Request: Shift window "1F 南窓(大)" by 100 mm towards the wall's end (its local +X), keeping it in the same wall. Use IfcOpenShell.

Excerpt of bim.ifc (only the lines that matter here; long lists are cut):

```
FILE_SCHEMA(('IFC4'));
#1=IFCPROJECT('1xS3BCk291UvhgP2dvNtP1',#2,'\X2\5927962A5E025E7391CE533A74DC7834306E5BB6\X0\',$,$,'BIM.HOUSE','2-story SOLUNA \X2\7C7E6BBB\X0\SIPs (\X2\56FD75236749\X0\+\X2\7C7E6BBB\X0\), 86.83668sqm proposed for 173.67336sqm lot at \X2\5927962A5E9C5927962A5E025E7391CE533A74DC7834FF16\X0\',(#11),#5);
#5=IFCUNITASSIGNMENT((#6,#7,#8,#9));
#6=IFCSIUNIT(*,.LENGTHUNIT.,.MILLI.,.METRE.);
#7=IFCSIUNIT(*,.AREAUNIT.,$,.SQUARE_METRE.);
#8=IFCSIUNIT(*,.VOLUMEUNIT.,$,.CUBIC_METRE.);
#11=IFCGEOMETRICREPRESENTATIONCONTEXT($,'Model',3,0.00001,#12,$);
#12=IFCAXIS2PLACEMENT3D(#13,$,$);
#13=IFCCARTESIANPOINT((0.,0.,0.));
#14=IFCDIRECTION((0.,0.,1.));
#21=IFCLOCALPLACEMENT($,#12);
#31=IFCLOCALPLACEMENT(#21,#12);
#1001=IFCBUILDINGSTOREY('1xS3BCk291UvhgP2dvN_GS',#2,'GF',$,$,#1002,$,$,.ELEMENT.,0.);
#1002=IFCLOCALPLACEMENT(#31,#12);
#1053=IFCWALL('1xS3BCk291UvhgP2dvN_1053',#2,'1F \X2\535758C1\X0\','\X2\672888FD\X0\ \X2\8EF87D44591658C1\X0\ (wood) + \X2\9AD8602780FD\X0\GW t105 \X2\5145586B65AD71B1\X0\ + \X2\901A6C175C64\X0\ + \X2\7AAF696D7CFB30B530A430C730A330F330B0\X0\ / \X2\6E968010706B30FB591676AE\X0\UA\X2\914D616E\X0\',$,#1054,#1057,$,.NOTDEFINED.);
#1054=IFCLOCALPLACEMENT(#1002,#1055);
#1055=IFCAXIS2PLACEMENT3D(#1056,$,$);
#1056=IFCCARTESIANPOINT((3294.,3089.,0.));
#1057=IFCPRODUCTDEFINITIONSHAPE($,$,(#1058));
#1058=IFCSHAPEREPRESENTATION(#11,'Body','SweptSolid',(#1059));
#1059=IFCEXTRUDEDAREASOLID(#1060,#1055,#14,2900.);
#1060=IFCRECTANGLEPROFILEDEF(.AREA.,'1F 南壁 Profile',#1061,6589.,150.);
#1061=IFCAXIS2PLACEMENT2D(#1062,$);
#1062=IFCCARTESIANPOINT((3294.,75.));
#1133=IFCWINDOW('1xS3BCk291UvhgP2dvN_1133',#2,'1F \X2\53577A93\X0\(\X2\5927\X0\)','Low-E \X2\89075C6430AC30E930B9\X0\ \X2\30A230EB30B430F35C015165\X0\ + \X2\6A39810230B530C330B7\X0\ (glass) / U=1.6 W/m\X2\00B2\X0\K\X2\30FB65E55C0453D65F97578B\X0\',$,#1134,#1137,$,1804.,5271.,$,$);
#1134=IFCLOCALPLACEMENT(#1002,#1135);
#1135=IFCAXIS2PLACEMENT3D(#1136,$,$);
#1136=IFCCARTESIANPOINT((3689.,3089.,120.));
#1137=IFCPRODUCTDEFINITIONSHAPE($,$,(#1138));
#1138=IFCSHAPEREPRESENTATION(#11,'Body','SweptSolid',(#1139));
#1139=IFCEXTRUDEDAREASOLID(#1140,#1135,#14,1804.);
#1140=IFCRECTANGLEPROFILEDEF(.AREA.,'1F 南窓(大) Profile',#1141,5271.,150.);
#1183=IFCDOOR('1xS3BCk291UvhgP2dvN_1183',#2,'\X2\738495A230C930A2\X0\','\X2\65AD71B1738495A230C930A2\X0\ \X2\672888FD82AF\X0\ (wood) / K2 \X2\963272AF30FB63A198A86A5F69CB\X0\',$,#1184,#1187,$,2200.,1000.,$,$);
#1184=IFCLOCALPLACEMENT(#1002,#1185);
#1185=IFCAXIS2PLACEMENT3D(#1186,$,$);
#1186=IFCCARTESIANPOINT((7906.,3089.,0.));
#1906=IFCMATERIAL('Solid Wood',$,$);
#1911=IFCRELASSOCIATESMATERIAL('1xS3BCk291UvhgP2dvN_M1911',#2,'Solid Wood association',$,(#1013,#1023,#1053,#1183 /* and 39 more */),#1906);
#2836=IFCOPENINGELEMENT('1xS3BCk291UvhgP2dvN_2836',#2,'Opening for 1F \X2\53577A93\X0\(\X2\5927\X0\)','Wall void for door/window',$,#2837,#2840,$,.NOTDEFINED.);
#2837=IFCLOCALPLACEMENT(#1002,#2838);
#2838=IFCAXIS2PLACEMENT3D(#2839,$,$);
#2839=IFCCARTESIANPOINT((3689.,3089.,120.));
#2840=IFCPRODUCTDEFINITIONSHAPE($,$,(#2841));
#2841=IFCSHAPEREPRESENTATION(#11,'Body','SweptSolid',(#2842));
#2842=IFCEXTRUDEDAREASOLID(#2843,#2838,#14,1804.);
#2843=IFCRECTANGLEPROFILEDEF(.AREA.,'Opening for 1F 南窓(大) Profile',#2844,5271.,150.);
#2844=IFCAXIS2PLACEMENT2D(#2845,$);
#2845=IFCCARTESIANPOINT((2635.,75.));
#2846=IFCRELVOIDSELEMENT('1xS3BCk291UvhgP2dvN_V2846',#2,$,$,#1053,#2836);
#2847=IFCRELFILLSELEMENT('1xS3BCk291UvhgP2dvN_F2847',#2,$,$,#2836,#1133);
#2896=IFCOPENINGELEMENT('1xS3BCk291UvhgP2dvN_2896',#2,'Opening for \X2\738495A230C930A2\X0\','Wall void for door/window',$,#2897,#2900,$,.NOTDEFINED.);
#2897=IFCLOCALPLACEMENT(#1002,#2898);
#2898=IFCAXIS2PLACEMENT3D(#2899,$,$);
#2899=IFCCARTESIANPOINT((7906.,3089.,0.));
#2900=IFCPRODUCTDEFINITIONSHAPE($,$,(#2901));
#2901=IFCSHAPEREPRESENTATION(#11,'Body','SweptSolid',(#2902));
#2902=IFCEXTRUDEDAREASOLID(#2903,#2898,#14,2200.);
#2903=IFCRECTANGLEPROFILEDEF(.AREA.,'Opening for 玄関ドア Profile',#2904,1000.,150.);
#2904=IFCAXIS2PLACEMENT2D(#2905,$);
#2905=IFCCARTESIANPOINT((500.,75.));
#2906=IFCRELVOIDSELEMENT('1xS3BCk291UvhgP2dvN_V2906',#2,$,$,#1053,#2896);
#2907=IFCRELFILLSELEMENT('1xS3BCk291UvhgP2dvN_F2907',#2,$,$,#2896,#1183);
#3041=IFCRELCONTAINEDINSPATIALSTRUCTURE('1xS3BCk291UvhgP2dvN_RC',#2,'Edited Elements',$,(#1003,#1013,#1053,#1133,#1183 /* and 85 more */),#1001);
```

```python
import ifcopenshell
import ifcopenshell.api.geometry
import ifcopenshell.util.placement

model = ifcopenshell.open("bim.ifc")

window = model.by_guid("1xS3BCk291UvhgP2dvN_1133")
opening = window.FillsVoids[0].RelatingOpeningElement
wall = opening.VoidsElements[0].RelatingBuildingElement

wall_matrix = ifcopenshell.util.placement.get_local_placement(wall.ObjectPlacement)
shift = wall_matrix[:3, 0] * 100.0
before = ifcopenshell.util.placement.get_local_placement(window.ObjectPlacement)[:3, 3].copy()

# The window is not placed relative to its opening, so move both.
for product in (opening, window):
    matrix = ifcopenshell.util.placement.get_local_placement(product.ObjectPlacement)
    matrix[:3, 3] += shift
    ifcopenshell.api.geometry.edit_object_placement(model, product=product, matrix=matrix, is_si=False)

after = ifcopenshell.util.placement.get_local_placement(window.ObjectPlacement)[:3, 3]
print("window moved by", (after - before).round(3) + 0.0)

model.write("bim_rev.ifc")
```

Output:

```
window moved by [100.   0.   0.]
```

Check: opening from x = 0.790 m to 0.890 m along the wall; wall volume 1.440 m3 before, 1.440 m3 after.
